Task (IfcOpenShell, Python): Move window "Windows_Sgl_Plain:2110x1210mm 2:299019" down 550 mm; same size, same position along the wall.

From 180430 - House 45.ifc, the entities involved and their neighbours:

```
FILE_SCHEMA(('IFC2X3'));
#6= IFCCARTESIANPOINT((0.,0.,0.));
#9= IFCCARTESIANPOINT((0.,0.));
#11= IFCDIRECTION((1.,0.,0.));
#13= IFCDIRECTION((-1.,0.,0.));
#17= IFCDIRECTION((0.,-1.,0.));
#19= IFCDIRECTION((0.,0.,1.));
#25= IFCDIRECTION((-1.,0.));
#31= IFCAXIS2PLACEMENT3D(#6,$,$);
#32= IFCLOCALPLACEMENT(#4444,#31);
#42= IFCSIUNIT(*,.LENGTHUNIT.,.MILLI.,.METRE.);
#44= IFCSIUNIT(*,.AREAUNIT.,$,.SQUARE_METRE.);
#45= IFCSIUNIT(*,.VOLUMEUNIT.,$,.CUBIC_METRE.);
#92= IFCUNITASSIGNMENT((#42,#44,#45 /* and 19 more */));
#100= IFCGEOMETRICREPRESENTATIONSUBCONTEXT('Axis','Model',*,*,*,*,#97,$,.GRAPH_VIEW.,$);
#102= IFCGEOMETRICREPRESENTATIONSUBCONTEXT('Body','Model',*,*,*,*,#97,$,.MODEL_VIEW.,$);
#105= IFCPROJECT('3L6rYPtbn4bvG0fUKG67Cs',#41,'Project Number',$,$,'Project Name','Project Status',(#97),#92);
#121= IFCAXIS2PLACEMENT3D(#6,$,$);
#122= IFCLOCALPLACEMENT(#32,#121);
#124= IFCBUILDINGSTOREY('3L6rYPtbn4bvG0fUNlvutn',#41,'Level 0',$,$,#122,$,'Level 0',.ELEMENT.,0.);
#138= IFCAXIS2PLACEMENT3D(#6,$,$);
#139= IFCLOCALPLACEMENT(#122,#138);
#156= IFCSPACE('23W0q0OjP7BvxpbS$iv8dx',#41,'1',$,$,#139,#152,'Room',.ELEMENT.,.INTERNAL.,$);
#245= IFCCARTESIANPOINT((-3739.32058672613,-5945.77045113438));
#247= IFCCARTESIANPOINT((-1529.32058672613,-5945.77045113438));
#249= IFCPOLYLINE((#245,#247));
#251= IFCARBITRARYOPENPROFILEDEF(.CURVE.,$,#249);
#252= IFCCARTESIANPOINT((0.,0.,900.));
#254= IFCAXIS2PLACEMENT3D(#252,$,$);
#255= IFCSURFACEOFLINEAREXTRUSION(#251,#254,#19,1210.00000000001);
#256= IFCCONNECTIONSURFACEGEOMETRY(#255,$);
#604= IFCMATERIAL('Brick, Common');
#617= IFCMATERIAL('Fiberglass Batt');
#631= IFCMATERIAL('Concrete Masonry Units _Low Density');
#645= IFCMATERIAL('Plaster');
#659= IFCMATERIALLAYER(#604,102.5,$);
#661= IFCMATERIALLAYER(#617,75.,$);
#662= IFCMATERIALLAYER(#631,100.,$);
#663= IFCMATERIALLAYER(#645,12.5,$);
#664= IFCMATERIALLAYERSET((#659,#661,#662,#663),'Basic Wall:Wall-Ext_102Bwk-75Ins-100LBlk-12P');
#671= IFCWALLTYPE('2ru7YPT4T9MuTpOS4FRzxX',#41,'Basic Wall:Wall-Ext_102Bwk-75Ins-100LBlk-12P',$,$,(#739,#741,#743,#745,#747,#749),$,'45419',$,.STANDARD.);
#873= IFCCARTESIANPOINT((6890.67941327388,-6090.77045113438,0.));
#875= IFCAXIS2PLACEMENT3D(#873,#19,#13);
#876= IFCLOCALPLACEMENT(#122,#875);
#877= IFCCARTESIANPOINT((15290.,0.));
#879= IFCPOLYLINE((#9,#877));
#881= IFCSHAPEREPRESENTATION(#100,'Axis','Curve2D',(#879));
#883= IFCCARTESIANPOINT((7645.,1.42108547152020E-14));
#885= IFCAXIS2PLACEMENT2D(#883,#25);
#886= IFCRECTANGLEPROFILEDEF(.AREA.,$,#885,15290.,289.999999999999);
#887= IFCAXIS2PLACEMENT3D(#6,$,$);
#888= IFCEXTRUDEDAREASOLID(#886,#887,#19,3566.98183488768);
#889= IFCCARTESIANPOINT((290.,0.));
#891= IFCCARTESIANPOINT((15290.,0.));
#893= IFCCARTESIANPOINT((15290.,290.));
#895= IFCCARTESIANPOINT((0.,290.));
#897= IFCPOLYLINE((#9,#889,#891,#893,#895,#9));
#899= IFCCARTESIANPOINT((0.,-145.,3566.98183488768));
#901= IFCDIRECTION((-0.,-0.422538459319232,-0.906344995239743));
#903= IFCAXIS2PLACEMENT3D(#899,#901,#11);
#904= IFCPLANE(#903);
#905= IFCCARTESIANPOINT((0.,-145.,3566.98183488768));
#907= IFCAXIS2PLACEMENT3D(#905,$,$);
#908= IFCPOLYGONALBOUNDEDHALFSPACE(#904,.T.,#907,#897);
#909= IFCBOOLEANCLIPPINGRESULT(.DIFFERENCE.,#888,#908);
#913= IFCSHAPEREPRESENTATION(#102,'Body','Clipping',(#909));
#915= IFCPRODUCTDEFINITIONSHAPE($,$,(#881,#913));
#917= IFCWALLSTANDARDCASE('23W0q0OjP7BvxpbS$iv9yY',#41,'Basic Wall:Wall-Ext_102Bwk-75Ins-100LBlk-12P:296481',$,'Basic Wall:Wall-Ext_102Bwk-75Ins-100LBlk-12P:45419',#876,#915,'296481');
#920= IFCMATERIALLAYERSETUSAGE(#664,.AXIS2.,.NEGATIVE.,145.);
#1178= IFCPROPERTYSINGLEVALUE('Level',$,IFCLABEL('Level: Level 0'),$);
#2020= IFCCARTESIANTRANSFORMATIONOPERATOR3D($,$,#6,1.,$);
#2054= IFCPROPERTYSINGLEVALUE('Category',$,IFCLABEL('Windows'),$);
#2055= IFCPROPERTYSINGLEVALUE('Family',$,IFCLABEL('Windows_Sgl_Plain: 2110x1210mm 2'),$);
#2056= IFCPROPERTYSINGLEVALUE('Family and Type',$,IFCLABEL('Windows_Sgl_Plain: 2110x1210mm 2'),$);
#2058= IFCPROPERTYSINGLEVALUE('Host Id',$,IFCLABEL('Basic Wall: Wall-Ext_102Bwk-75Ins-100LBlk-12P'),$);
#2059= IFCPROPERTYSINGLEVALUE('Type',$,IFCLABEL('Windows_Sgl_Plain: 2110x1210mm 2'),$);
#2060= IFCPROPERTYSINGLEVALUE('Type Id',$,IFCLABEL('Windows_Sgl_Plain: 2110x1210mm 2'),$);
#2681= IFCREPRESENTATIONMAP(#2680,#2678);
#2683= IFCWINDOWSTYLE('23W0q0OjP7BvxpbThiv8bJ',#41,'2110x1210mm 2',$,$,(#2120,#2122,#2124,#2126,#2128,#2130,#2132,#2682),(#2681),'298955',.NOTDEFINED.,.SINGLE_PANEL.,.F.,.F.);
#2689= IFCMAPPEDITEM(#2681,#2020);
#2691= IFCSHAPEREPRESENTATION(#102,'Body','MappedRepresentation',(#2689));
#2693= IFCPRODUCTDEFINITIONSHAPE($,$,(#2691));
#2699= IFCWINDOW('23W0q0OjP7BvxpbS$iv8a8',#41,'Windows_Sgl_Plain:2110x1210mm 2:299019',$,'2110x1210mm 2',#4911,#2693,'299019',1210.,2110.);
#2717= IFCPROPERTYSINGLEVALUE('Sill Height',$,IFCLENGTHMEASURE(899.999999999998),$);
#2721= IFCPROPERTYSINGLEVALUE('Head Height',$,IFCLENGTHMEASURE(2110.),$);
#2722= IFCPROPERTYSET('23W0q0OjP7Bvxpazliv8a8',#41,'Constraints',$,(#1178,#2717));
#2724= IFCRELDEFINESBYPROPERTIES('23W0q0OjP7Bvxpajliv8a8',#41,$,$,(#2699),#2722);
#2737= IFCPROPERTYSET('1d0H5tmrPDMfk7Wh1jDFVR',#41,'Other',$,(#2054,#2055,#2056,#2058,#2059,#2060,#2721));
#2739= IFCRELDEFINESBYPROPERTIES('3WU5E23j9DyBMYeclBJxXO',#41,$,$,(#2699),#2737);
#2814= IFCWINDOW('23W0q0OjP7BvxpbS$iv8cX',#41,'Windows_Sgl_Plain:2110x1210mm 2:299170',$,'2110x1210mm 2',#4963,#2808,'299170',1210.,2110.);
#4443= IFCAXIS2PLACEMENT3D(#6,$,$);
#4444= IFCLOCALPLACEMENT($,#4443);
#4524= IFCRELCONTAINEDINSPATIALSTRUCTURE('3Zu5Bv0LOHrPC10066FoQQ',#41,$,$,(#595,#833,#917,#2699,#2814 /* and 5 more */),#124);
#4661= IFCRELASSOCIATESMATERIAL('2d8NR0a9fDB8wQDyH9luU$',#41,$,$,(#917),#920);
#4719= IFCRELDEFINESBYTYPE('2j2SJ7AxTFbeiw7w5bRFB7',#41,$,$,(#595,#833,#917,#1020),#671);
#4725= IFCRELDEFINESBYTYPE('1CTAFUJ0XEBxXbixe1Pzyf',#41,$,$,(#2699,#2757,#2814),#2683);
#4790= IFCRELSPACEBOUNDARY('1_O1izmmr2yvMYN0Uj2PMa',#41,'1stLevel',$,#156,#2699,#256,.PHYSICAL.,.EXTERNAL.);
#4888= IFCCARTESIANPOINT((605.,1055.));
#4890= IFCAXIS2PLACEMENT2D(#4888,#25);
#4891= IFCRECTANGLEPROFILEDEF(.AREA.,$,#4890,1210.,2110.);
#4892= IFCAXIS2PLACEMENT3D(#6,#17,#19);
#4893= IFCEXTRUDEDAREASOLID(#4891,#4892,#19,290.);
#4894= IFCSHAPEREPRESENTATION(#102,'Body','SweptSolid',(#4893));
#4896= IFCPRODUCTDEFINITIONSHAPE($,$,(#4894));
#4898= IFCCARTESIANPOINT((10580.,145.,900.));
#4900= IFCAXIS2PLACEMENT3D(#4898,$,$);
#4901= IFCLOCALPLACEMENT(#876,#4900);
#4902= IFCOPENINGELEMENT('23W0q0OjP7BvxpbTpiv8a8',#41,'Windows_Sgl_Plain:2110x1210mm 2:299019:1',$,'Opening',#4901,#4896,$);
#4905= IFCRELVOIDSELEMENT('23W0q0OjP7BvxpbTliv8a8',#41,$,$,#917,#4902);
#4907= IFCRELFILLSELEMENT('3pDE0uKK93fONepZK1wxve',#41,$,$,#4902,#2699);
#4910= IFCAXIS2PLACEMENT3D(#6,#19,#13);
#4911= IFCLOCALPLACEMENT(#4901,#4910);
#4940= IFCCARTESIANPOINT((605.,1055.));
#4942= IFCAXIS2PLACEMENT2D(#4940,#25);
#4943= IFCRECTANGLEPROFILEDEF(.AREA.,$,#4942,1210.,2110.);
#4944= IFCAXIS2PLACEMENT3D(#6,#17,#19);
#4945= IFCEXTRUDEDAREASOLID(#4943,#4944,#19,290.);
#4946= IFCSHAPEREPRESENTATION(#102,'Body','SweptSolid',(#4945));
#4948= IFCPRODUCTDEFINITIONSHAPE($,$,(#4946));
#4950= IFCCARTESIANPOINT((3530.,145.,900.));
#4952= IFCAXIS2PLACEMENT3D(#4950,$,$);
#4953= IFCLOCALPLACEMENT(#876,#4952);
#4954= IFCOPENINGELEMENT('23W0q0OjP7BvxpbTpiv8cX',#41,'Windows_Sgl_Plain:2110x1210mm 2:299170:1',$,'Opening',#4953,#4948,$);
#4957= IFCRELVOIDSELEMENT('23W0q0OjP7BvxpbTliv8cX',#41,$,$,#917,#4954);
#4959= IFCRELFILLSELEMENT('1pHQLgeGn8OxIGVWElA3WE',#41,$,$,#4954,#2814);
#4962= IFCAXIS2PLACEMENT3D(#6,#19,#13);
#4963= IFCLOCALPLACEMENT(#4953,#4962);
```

```python
import numpy as np
import ifcopenshell
import ifcopenshell.api.geometry
import ifcopenshell.api.pset
import ifcopenshell.util.element
import ifcopenshell.util.placement
import ifcopenshell.util.unit

model = ifcopenshell.open("180430 - House 45.ifc")
unit_scale = ifcopenshell.util.unit.calculate_unit_scale(model)

window = model.by_guid("23W0q0OjP7BvxpbS$iv8a8")
opening = window.FillsVoids[0].RelatingOpeningElement
dz = -0.55 / unit_scale

shift = np.array([0.0, 0.0, dz])
# The window is placed relative to its opening, so it follows when the opening moves.
matrix = ifcopenshell.util.placement.get_local_placement(opening.ObjectPlacement)
matrix[:3, 3] += shift
ifcopenshell.api.geometry.edit_object_placement(
    model, product=opening, matrix=matrix, is_si=False, should_transform_children=True
)

# Space boundary surfaces are stored in each space's coordinates; move them too.
for rel in window.ProvidesBoundaries:
    if not rel.ConnectionGeometry:
        continue
    surface = rel.ConnectionGeometry.SurfaceOnRelatingElement
    space_matrix = ifcopenshell.util.placement.get_local_placement(rel.RelatingSpace.ObjectPlacement)
    point = np.array(surface.Position.Location.Coordinates) + space_matrix[:3, :3].T @ shift
    surface.Position = model.createIfcAxis2Placement3D(
        model.createIfcCartesianPoint(point.tolist()), surface.Position.Axis, surface.Position.RefDirection
    )

# Keep the stored heights in step.
pset = model.by_id(ifcopenshell.util.element.get_pset(window, "Constraints", should_inherit=False)["id"])
ifcopenshell.api.pset.edit_pset(model, pset=pset, properties={
    "Sill Height": model.create_entity("IfcLengthMeasure", ifcopenshell.util.element.get_pset(window, "Constraints", "Sill Height") + dz),
})
pset = model.by_id(ifcopenshell.util.element.get_pset(window, "Other", should_inherit=False)["id"])
ifcopenshell.api.pset.edit_pset(model, pset=pset, properties={
    "Head Height": model.create_entity("IfcLengthMeasure", ifcopenshell.util.element.get_pset(window, "Other", "Head Height") + dz),
})

print(f"moved by {dz * unit_scale:+.3f} m")

model.write("180430 - House 45_edited.ifc")
```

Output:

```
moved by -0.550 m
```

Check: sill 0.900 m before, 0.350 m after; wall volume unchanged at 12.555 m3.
